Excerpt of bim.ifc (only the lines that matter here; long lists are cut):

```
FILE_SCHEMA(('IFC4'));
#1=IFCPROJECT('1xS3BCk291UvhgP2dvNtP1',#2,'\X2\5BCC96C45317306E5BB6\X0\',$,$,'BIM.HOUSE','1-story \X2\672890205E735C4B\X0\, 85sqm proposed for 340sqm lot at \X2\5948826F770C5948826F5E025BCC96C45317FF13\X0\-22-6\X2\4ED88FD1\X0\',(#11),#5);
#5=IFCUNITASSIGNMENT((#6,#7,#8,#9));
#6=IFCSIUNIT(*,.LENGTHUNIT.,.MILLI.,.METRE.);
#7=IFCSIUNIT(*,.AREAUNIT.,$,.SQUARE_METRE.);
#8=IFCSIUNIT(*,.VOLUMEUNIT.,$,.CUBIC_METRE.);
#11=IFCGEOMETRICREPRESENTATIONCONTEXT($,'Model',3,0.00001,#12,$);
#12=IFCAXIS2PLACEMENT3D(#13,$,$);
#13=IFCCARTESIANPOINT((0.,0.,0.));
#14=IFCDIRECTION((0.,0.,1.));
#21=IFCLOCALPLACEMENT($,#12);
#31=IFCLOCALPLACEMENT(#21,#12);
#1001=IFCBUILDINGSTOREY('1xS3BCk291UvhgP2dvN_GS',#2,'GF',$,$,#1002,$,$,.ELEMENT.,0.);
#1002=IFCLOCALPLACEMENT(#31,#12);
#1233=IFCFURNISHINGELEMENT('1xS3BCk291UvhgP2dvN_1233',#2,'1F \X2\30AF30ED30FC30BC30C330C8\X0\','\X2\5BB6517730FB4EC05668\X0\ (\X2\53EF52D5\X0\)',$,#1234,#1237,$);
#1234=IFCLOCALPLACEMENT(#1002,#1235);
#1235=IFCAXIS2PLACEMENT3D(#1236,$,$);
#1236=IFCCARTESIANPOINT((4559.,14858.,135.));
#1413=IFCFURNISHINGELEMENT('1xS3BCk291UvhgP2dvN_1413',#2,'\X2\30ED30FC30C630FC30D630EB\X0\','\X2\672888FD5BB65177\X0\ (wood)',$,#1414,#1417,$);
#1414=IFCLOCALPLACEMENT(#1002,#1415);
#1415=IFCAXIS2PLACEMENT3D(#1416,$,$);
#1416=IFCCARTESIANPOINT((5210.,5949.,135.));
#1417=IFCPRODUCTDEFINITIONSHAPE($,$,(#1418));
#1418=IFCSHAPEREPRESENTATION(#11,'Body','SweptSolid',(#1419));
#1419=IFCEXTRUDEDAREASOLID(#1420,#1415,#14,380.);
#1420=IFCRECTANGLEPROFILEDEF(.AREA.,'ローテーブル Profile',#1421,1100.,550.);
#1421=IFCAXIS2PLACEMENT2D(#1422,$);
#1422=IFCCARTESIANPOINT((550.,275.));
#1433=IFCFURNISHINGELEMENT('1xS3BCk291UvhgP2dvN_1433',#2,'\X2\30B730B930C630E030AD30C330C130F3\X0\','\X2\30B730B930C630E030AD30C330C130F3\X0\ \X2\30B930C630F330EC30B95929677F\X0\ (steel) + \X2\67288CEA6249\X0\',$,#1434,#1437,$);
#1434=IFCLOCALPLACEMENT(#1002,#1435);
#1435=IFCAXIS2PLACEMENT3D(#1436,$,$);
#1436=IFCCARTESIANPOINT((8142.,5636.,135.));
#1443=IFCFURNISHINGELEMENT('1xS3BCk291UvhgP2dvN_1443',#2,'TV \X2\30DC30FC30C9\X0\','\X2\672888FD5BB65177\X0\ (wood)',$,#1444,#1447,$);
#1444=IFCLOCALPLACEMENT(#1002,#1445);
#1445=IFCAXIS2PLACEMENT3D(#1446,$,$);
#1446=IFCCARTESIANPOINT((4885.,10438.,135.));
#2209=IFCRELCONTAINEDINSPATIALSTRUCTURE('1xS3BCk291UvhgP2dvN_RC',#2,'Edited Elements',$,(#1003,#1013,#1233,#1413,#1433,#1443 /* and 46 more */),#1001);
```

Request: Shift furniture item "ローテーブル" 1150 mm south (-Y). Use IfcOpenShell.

```python
import ifcopenshell
import ifcopenshell.api.geometry
import ifcopenshell.util.placement
import ifcopenshell.util.unit

model = ifcopenshell.open("bim.ifc")
unit_scale = ifcopenshell.util.unit.calculate_unit_scale(model)

item = model.by_guid("1xS3BCk291UvhgP2dvN_1413")
matrix = ifcopenshell.util.placement.get_local_placement(item.ObjectPlacement)
matrix[1, 3] -= 1.15 / unit_scale
ifcopenshell.api.geometry.edit_object_placement(model, product=item, matrix=matrix, is_si=False)

print(ifcopenshell.util.placement.get_local_placement(item.ObjectPlacement).round(3) + 0.0)

model.write("bim_updated.ifc")
```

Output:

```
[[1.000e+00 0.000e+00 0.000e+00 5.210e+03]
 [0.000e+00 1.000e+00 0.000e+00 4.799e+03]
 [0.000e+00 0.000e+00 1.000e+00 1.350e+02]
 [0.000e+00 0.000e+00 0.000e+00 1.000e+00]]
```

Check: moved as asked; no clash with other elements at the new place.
